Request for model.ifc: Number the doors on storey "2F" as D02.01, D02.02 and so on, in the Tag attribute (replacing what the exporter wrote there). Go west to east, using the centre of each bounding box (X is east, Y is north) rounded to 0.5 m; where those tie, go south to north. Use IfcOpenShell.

First a look at what the model holds.

```python
import ifcopenshell
import ifcopenshell.util.element
import ifcopenshell.util.placement

model = ifcopenshell.open("model.ifc")
print(model.schema)
storey = next(s for s in model.by_type("IfcBuildingStorey") if s.Name == "2F")
doors = [e for e in ifcopenshell.util.element.get_decomposition(storey) if e.is_a("IfcDoor")]
for e in sorted(doors, key=lambda e: e.id()):
    origin = ifcopenshell.util.placement.get_local_placement(e.ObjectPlacement)[:3, 3]
    print(e.id(), e.Tag, e.Name, origin.round(2) + 0.0, sep=" | ")
```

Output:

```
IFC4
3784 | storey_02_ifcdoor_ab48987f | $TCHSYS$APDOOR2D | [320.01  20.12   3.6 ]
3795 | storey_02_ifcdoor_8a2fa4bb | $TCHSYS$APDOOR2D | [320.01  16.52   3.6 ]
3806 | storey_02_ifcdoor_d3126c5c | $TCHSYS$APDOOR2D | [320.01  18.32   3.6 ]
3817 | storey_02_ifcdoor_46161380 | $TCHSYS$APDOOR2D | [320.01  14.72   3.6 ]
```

```python
import ifcopenshell
import ifcopenshell.geom
import ifcopenshell.util.element
import ifcopenshell.util.shape

model = ifcopenshell.open("model.ifc")
settings = ifcopenshell.geom.settings()
settings.set("use-world-coords", True)


def centre(element):
    shape = ifcopenshell.geom.create_shape(settings, element)
    return ifcopenshell.util.shape.get_bbox_centroid(shape.geometry)


storey = next(s for s in model.by_type("IfcBuildingStorey") if s.Name == "2F")
doors = [e for e in ifcopenshell.util.element.get_decomposition(storey) if e.is_a("IfcDoor")]

# Insertion points can sit at a corner or the storey origin, so sort by the geometry (in metres).
centres = {e: centre(e) for e in doors}
doors.sort(key=lambda e: (round(centres[e][0] / 0.5), centres[e][1]))

for i, e in enumerate(doors, start=1):
    number = f"D02.{i:02d}"
    e.Tag = number
    print(e.id(), number)

model.write("model-out.ifc")
```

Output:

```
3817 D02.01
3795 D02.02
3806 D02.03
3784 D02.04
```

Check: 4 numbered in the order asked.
